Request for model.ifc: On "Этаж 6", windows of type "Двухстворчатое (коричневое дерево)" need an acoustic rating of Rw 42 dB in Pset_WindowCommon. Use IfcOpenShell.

First a look at what the model holds.

```python
import ifcopenshell
import ifcopenshell.util.element

model = ifcopenshell.open("model.ifc")
print(model.schema)
storey = next(s for s in model.by_type("IfcBuildingStorey") if s.Name == "Этаж 6")
windows = [e for e in ifcopenshell.util.element.get_decomposition(storey) if e.is_a("IfcWindow")]
seen = {}
for e in windows:
    element_type = ifcopenshell.util.element.get_type(e)
    key = (element_type.Name if element_type != e and element_type else None, ifcopenshell.util.element.get_pset(e, "Pset_WindowCommon", "AcousticRating"))
    seen[key] = seen.get(key, 0) + 1
for (name, value), count in sorted(seen.items(), key=str):
    print(count, "x", name, "|", value)
```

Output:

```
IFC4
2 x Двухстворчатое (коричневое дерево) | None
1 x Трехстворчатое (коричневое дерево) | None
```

```python
import ifcopenshell
import ifcopenshell.api.pset
import ifcopenshell.util.element

model = ifcopenshell.open("model.ifc")

storey = next(s for s in model.by_type("IfcBuildingStorey") if s.Name == "Этаж 6")
windows = [e for e in ifcopenshell.util.element.get_decomposition(storey) if e.is_a("IfcWindow")]

count = 0
for e in windows:
    element_type = ifcopenshell.util.element.get_type(e)
    if element_type in (None, e) or element_type.Name != "Двухстворчатое (коричневое дерево)":
        continue
    # add_pset returns the element's existing set when there is one.
    pset = ifcopenshell.api.pset.add_pset(model, product=e, name="Pset_WindowCommon")
    ifcopenshell.api.pset.edit_pset(model, pset=pset, properties={"AcousticRating": "Rw 42 dB"})
    count += 1

print(count, "windows updated")

model.write("model_edited.ifc")
```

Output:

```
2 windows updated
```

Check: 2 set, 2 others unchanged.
